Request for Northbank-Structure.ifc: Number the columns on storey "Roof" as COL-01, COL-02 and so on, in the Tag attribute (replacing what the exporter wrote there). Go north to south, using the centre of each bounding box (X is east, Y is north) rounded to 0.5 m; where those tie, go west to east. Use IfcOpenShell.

First a look at what the model holds.

```python
import ifcopenshell
import ifcopenshell.util.element
import ifcopenshell.util.placement

model = ifcopenshell.open("Northbank-Structure.ifc")
print(model.schema)
storey = next(s for s in model.by_type("IfcBuildingStorey") if s.Name == "Roof")
columns = [e for e in ifcopenshell.util.element.get_decomposition(storey) if e.is_a("IfcColumn")]
for e in sorted(columns, key=lambda e: e.id()):
    origin = ifcopenshell.util.placement.get_local_placement(e.ObjectPlacement)[:3, 3]
    print(e.id(), e.Tag, e.Name, origin.round(2) + 0.0, sep=" | ")
```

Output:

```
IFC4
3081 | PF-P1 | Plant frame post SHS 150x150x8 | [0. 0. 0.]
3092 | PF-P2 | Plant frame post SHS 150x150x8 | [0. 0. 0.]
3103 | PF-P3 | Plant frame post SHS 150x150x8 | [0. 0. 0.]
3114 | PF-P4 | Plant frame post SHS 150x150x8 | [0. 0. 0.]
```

```python
import ifcopenshell
import ifcopenshell.geom
import ifcopenshell.util.element
import ifcopenshell.util.shape

model = ifcopenshell.open("Northbank-Structure.ifc")
settings = ifcopenshell.geom.settings()
settings.set("use-world-coords", True)


def centre(element):
    shape = ifcopenshell.geom.create_shape(settings, element)
    return ifcopenshell.util.shape.get_bbox_centroid(shape.geometry)


storey = next(s for s in model.by_type("IfcBuildingStorey") if s.Name == "Roof")
columns = [e for e in ifcopenshell.util.element.get_decomposition(storey) if e.is_a("IfcColumn")]

# Insertion points can sit at a corner or the storey origin, so sort by the geometry (in metres).
centres = {e: centre(e) for e in columns}
columns.sort(key=lambda e: (-round(centres[e][1] / 0.5), centres[e][0]))

for i, e in enumerate(columns, start=1):
    number = f"COL-{i:02d}"
    e.Tag = number
    print(e.id(), number)

model.write("Northbank-Structure_v2.ifc")
```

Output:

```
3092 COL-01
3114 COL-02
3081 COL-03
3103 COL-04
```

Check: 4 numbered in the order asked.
